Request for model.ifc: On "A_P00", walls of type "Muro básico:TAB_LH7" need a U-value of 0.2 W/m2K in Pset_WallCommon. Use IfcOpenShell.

First a look at what the model holds.

```python
import ifcopenshell
import ifcopenshell.util.element

model = ifcopenshell.open("model.ifc")
print(model.schema)
storey = next(s for s in model.by_type("IfcBuildingStorey") if s.Name == "A_P00")
walls = [e for e in ifcopenshell.util.element.get_decomposition(storey) if e.is_a("IfcWall")]
seen = {}
for e in walls:
    element_type = ifcopenshell.util.element.get_type(e)
    key = (element_type.Name if element_type != e and element_type else None, ifcopenshell.util.element.get_pset(e, "Pset_WallCommon", "ThermalTransmittance"))
    seen[key] = seen.get(key, 0) + 1
for (name, value), count in sorted(seen.items(), key=str):
    print(count, "x", name, "|", value)
```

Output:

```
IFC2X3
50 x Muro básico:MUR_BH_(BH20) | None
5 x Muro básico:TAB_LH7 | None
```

```python
import ifcopenshell
import ifcopenshell.api.pset
import ifcopenshell.util.element

model = ifcopenshell.open("model.ifc")

storey = next(s for s in model.by_type("IfcBuildingStorey") if s.Name == "A_P00")
walls = [e for e in ifcopenshell.util.element.get_decomposition(storey) if e.is_a("IfcWall")]

count = 0
for e in walls:
    element_type = ifcopenshell.util.element.get_type(e)
    if element_type in (None, e) or element_type.Name != "Muro básico:TAB_LH7":
        continue
    # add_pset returns the element's existing set when there is one.
    pset = ifcopenshell.api.pset.add_pset(model, product=e, name="Pset_WallCommon")
    ifcopenshell.api.pset.edit_pset(model, pset=pset, properties={"ThermalTransmittance": 0.2})
    count += 1

print(count, "walls updated")

model.write("model_v2.ifc")
```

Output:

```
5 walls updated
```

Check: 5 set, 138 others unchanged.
